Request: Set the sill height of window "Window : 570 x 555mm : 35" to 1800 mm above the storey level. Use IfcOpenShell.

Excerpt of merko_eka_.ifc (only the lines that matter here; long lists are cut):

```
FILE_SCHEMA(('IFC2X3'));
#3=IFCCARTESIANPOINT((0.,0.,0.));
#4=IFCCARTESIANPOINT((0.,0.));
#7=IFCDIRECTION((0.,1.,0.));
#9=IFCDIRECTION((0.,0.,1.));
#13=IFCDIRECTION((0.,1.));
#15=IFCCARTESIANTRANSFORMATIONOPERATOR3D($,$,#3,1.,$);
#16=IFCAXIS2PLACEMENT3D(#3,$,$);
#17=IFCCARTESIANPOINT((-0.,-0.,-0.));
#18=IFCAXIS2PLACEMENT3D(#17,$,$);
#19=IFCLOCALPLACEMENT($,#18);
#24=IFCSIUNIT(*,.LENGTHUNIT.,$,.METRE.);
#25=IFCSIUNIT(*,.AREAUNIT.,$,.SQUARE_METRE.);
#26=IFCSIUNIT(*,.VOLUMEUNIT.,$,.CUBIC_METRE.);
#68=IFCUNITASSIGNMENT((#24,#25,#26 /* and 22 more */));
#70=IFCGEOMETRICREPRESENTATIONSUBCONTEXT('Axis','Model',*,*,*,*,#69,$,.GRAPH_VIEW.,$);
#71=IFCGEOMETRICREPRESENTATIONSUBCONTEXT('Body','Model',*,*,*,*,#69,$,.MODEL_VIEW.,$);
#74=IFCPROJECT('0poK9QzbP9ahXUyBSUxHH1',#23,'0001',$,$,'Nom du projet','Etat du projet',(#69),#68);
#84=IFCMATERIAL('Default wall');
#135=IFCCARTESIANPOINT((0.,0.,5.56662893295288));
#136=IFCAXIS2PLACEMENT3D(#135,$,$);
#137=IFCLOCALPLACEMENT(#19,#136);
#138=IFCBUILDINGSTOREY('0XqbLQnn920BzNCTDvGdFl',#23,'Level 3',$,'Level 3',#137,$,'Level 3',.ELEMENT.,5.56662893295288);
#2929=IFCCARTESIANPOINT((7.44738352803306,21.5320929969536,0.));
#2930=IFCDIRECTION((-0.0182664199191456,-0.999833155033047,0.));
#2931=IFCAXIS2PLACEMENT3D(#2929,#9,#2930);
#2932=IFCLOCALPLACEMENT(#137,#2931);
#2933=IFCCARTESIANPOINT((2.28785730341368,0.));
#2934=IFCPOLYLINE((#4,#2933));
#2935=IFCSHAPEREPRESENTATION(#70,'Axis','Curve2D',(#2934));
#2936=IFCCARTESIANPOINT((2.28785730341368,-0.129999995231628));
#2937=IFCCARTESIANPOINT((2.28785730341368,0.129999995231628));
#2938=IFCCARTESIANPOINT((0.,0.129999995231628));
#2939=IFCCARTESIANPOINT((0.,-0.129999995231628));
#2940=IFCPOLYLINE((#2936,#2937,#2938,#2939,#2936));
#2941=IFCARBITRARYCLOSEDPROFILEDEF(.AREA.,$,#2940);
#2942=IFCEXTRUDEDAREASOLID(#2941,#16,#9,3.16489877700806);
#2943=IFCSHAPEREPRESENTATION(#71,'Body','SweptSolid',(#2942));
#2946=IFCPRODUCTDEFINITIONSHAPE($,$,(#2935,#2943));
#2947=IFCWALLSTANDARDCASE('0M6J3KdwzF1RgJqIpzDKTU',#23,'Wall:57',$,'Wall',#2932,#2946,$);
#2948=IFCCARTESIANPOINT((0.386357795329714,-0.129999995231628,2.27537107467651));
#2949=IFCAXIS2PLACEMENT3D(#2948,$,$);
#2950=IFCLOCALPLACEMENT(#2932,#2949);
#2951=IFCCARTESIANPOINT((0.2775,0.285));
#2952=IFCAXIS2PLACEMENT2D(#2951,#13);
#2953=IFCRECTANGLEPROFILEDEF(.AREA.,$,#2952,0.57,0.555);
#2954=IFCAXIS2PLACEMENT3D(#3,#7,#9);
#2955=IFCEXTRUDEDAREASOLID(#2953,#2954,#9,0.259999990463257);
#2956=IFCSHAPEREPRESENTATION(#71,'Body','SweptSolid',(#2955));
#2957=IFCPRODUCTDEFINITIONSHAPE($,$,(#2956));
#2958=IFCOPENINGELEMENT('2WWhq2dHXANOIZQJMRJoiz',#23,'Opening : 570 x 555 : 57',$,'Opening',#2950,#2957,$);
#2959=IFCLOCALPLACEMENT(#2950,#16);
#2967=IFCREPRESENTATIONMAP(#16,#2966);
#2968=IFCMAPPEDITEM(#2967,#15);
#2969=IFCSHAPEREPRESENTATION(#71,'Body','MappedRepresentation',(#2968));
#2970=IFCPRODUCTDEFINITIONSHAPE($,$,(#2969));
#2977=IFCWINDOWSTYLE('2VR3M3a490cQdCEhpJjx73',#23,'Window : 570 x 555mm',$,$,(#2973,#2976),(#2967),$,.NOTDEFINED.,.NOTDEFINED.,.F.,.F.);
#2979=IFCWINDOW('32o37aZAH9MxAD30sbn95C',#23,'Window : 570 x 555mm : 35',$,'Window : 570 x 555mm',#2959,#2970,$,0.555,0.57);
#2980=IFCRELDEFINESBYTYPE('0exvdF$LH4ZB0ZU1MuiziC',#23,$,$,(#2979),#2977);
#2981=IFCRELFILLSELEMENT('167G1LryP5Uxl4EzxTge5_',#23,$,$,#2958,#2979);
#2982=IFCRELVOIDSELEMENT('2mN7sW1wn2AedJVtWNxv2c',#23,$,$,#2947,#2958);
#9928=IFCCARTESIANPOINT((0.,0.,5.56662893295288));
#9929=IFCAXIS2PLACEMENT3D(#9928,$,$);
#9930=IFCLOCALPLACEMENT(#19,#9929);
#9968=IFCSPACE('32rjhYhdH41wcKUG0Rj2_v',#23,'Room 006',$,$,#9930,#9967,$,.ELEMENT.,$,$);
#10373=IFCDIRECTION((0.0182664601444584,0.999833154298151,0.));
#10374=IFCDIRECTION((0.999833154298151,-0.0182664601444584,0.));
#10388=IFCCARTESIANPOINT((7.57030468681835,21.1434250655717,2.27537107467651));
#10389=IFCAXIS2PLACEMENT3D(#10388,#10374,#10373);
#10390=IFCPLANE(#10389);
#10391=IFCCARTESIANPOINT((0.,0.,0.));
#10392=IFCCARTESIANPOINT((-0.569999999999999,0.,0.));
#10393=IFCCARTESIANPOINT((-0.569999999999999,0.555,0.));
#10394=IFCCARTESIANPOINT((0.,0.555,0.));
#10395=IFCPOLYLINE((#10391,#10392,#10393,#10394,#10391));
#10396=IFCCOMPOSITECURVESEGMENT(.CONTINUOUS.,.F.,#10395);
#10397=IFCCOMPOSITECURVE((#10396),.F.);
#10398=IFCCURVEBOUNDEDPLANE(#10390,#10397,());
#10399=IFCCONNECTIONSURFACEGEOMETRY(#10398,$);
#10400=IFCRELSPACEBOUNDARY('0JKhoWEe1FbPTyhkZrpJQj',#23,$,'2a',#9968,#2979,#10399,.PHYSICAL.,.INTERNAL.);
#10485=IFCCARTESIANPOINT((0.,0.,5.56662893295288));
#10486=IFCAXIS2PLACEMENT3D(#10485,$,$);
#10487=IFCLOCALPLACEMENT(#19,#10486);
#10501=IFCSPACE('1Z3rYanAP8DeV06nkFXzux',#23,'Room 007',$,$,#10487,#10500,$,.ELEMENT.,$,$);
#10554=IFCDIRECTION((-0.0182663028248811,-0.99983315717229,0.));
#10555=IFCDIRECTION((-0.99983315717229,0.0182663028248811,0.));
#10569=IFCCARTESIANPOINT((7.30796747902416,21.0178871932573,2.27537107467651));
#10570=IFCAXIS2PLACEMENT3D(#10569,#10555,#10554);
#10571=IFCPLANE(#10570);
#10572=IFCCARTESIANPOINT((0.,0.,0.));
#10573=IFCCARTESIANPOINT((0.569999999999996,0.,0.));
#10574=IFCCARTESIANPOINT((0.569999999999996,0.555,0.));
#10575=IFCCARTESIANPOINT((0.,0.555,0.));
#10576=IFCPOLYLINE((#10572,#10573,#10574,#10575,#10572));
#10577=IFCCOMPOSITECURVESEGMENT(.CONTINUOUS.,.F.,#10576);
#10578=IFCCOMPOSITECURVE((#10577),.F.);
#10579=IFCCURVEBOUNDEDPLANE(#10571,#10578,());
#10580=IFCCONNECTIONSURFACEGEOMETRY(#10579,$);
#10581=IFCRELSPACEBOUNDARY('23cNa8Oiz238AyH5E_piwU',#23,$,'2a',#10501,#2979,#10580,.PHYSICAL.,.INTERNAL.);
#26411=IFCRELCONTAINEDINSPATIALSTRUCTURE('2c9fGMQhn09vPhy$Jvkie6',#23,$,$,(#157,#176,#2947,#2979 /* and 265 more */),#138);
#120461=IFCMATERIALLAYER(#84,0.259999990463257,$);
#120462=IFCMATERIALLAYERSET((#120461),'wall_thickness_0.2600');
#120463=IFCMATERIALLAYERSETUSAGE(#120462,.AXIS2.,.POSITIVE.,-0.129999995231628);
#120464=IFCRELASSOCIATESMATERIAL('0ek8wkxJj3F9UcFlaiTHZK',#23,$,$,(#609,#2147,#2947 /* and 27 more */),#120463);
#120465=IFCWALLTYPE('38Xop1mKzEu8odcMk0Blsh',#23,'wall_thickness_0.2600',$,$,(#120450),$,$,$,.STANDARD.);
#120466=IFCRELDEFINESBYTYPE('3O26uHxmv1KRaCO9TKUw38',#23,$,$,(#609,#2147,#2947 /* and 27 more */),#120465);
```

```python
import numpy as np
import ifcopenshell
import ifcopenshell.api.geometry
import ifcopenshell.geom
import ifcopenshell.util.element
import ifcopenshell.util.placement
import ifcopenshell.util.shape
import ifcopenshell.util.unit

model = ifcopenshell.open("merko_eka_.ifc")
unit_scale = ifcopenshell.util.unit.calculate_unit_scale(model)

window = model.by_id(2979)
opening = window.FillsVoids[0].RelatingOpeningElement
storey = ifcopenshell.util.element.get_container(window, ifc_class="IfcBuildingStorey")
level = ifcopenshell.util.placement.get_local_placement(storey.ObjectPlacement)[2, 3]

# The opening's origin need not be at the sill, so measure its lowest point.
shape = ifcopenshell.geom.create_shape(ifcopenshell.geom.settings(), opening)
bottom = ifcopenshell.util.shape.get_shape_bottom_elevation(shape, shape.geometry) / unit_scale
dz = level + 1.8 - bottom

shift = np.array([0.0, 0.0, dz])
# The window is placed relative to its opening, so it follows when the opening moves.
matrix = ifcopenshell.util.placement.get_local_placement(opening.ObjectPlacement)
matrix[:3, 3] += shift
ifcopenshell.api.geometry.edit_object_placement(
    model, product=opening, matrix=matrix, is_si=False, should_transform_children=True
)

# Space boundary surfaces are stored in each space's coordinates; move them too.
for rel in window.ProvidesBoundaries:
    if not rel.ConnectionGeometry:
        continue
    surface = rel.ConnectionGeometry.SurfaceOnRelatingElement.BasisSurface
    space_matrix = ifcopenshell.util.placement.get_local_placement(rel.RelatingSpace.ObjectPlacement)
    point = np.array(surface.Position.Location.Coordinates) + space_matrix[:3, :3].T @ shift
    surface.Position = model.createIfcAxis2Placement3D(
        model.createIfcCartesianPoint(point.tolist()), surface.Position.Axis, surface.Position.RefDirection
    )

print(f"moved by {dz * unit_scale:+.3f} m")

model.write("merko_eka__updated.ifc")
```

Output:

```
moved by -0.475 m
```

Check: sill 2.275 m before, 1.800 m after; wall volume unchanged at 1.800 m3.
